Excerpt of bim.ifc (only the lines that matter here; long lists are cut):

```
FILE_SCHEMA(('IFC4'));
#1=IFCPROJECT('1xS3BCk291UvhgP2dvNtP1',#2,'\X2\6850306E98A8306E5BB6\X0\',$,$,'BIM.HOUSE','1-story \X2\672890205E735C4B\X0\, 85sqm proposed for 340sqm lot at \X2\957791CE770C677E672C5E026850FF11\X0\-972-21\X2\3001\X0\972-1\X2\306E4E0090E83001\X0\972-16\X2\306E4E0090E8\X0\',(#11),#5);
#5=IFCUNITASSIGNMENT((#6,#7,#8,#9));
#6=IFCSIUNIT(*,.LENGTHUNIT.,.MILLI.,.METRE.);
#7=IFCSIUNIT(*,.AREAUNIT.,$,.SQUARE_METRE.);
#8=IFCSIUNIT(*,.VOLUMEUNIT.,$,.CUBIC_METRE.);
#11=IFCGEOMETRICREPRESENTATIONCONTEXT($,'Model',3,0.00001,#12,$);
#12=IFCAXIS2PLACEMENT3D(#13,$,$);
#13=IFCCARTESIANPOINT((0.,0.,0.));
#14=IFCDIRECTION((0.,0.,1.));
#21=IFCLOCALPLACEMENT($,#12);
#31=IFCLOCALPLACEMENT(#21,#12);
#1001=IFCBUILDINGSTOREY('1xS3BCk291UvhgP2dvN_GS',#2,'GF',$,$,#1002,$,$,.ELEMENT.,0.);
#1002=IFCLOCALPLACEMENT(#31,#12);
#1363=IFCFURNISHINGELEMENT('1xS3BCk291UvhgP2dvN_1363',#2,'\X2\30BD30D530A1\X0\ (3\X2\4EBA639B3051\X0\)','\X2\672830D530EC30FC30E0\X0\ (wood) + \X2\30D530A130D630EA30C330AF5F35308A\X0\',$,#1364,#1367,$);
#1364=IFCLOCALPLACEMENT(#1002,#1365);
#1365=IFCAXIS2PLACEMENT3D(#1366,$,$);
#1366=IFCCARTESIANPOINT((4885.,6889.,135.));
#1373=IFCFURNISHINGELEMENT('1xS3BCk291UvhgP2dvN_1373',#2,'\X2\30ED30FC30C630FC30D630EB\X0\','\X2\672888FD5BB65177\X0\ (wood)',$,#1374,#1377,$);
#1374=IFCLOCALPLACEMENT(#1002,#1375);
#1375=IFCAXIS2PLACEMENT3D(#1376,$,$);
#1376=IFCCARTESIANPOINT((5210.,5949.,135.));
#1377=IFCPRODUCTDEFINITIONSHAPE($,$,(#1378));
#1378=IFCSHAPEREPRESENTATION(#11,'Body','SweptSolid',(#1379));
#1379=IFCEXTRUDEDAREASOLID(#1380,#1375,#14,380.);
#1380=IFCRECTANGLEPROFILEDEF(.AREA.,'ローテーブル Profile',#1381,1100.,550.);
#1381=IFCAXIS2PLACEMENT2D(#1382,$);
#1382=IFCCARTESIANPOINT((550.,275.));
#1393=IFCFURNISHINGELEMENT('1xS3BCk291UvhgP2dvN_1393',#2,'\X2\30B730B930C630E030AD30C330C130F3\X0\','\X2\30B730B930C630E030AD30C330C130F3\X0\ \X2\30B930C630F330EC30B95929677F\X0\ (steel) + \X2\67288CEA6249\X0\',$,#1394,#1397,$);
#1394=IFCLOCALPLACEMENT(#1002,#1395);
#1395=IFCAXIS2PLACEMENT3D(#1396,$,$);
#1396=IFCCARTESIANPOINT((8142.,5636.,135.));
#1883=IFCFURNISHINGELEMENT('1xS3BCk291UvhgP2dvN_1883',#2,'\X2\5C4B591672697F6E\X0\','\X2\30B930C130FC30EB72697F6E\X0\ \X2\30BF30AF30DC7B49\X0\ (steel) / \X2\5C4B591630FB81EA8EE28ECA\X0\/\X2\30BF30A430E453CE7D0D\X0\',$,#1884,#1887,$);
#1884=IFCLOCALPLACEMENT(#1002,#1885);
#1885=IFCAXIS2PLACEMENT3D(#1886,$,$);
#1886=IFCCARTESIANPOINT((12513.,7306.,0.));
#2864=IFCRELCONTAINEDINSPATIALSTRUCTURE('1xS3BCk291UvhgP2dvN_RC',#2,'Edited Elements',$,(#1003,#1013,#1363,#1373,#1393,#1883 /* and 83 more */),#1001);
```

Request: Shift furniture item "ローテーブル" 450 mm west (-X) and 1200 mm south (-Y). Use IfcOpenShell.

```python
import ifcopenshell
import ifcopenshell.api.geometry
import ifcopenshell.util.placement
import ifcopenshell.util.unit

model = ifcopenshell.open("bim.ifc")
unit_scale = ifcopenshell.util.unit.calculate_unit_scale(model)

item = model.by_id(1373)
matrix = ifcopenshell.util.placement.get_local_placement(item.ObjectPlacement)
matrix[0, 3] -= 0.45 / unit_scale
matrix[1, 3] -= 1.2 / unit_scale
ifcopenshell.api.geometry.edit_object_placement(model, product=item, matrix=matrix, is_si=False)

print(ifcopenshell.util.placement.get_local_placement(item.ObjectPlacement).round(3) + 0.0)

model.write("bim_edited.ifc")
```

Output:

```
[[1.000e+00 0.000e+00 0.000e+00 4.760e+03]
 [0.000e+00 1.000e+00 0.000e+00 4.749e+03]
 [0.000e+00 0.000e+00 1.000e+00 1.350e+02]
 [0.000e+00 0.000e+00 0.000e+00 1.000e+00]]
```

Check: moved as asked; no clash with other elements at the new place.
